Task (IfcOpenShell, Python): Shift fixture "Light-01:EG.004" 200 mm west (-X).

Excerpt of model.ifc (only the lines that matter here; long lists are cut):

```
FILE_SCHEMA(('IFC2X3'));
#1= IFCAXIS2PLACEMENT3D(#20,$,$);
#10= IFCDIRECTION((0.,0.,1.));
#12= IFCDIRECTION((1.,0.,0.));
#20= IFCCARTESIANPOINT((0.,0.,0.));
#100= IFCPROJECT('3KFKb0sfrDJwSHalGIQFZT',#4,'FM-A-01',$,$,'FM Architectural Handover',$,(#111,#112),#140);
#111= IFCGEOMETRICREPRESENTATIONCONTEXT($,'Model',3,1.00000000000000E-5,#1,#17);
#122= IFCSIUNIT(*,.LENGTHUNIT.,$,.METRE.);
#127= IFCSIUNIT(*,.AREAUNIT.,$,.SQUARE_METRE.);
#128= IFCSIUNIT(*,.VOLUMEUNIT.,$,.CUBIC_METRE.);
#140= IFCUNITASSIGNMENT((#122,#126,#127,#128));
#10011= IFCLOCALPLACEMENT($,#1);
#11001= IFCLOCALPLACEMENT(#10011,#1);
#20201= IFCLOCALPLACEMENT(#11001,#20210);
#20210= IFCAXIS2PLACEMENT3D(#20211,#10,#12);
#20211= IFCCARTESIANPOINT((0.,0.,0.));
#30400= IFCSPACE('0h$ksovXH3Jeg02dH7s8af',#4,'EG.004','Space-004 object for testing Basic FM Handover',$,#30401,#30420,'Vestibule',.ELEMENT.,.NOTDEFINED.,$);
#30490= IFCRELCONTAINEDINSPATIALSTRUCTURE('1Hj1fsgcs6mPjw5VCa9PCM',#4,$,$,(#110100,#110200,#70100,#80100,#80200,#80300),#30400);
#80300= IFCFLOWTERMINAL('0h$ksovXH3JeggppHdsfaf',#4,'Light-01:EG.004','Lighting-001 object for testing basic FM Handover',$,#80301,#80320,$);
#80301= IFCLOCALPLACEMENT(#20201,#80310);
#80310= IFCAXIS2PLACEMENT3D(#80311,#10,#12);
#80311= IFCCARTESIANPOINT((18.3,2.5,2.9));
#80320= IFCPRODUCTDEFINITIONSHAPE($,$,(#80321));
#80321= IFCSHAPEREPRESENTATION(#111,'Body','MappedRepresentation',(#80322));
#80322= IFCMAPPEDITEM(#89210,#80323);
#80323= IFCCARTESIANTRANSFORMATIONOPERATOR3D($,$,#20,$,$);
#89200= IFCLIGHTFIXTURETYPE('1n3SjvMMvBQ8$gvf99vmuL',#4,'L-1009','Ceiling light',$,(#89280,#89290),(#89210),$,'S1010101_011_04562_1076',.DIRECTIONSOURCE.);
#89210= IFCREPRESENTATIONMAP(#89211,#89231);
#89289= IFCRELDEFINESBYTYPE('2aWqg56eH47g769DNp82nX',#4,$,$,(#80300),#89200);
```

```python
import ifcopenshell
import ifcopenshell.api.geometry
import ifcopenshell.util.placement

model = ifcopenshell.open("model.ifc")

item = model.by_id(80300)
matrix = ifcopenshell.util.placement.get_local_placement(item.ObjectPlacement)
matrix[0, 3] -= 0.2
ifcopenshell.api.geometry.edit_object_placement(model, product=item, matrix=matrix, is_si=False)

print(ifcopenshell.util.placement.get_local_placement(item.ObjectPlacement).round(3) + 0.0)

model.write("model_edited.ifc")
```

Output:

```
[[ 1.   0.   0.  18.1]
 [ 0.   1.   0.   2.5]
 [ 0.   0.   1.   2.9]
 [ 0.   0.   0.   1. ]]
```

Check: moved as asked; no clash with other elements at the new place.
